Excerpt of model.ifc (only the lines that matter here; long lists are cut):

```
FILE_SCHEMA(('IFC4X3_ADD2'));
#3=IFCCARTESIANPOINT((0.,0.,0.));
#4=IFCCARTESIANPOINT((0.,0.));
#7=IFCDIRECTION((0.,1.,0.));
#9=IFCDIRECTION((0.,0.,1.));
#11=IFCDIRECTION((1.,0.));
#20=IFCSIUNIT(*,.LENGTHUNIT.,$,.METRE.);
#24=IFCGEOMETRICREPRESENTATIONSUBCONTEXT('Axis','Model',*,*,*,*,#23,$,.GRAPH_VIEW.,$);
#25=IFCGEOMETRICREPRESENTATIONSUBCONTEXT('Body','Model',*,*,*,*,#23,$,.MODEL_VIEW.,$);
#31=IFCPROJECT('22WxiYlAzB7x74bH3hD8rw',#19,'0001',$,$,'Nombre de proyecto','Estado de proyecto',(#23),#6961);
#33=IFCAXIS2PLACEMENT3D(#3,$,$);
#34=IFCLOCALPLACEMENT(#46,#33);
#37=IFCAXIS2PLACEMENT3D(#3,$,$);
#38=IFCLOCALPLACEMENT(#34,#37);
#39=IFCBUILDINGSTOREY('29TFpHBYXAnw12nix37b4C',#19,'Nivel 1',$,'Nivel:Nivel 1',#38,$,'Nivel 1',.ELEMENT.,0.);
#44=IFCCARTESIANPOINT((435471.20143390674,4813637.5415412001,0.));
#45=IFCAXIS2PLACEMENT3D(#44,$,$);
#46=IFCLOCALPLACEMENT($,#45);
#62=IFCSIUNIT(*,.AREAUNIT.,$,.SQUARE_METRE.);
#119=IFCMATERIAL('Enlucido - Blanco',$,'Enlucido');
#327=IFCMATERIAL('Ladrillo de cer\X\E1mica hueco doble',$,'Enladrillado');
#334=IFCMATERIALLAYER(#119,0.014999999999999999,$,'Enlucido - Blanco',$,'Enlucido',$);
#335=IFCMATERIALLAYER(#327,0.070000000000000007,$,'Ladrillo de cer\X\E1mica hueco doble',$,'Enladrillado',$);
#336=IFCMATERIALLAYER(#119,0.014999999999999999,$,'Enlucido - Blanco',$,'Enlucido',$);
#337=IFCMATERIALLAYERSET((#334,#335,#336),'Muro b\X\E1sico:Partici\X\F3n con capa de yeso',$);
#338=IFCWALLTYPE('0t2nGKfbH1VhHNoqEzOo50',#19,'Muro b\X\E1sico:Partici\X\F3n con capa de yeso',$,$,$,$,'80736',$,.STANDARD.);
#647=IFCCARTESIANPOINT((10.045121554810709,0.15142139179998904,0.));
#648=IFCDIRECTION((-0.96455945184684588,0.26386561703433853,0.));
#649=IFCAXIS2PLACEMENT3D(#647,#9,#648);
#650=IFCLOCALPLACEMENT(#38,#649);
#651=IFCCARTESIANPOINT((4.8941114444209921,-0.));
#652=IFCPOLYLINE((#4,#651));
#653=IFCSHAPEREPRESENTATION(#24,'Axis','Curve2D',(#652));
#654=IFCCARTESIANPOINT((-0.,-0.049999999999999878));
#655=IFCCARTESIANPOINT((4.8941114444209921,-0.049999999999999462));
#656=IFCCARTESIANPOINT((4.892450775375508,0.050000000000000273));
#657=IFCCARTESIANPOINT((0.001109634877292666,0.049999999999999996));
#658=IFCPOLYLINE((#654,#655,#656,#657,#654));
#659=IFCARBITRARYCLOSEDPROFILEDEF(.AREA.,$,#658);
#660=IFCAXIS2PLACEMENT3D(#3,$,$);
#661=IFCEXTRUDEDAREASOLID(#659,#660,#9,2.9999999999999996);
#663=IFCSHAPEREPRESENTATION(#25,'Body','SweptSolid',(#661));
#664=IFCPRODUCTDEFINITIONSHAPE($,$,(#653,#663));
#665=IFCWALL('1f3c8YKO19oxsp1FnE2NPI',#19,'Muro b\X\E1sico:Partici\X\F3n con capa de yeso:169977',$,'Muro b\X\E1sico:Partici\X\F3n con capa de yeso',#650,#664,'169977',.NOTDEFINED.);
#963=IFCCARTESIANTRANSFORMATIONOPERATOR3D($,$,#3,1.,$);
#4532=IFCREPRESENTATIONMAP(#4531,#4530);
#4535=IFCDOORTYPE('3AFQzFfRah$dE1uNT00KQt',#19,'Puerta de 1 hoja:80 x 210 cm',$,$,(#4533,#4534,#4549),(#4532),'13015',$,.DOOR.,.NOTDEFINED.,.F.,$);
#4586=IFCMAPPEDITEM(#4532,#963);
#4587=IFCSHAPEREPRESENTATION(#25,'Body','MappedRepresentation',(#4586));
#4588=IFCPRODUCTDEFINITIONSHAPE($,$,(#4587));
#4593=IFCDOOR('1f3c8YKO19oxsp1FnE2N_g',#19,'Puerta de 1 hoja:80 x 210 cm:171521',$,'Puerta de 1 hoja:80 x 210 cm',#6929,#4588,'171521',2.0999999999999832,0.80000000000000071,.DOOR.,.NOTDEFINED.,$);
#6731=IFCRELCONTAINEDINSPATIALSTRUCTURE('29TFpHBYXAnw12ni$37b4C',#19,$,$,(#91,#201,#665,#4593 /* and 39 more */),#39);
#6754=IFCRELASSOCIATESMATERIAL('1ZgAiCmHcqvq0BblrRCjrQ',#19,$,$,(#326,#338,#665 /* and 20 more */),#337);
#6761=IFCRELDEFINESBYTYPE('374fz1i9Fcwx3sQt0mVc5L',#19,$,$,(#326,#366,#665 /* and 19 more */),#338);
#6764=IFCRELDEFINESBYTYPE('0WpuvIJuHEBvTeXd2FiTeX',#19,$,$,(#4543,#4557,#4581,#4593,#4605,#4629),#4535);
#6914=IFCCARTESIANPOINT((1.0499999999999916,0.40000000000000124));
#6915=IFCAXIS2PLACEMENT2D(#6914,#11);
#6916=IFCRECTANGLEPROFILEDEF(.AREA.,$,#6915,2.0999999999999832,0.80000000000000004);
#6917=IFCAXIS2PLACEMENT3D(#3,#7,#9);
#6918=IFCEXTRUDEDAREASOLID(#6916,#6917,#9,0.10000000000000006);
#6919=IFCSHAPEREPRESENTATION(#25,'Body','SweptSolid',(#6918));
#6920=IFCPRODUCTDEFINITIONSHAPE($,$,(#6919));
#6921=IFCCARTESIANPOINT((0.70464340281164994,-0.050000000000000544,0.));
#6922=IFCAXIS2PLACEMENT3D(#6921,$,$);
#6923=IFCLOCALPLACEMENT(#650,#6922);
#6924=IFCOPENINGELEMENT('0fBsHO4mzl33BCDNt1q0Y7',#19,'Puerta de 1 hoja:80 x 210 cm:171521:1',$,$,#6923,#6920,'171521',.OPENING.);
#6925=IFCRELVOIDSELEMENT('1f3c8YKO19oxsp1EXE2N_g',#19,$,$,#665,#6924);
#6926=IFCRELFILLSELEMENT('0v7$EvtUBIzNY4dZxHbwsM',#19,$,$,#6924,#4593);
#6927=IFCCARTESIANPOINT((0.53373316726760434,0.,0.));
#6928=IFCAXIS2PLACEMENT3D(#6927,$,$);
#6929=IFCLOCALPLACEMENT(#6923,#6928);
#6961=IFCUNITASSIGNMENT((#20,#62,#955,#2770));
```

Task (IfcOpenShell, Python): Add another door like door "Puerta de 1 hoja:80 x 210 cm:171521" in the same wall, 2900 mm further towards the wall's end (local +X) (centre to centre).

```python
import ifcopenshell
import ifcopenshell.api.feature
import ifcopenshell.api.geometry
import ifcopenshell.api.root
import ifcopenshell.geom
import ifcopenshell.util.element
import ifcopenshell.util.placement
import ifcopenshell.util.shape

model = ifcopenshell.open("model.ifc")
settings = ifcopenshell.geom.settings()


def volume(element):
    """Net volume in cubic metres, openings subtracted."""
    shape = ifcopenshell.geom.create_shape(settings, element)
    return ifcopenshell.util.shape.get_volume(shape.geometry)


def reuse_history(source, copy):
    """copy_class also copies each property set's owner history, people and application; keep the originals."""
    for rel in copy.IsDefinedBy:
        if rel.is_a("IfcRelDefinesByProperties") and (history := rel.RelatingPropertyDefinition.OwnerHistory):
            rel.RelatingPropertyDefinition.OwnerHistory = source.OwnerHistory
            ifcopenshell.util.element.remove_deep2(model, history)


door = model.by_id(4593)
opening = door.FillsVoids[0].RelatingOpeningElement
wall = opening.VoidsElements[0].RelatingBuildingElement
before = volume(wall)
shift = ifcopenshell.util.placement.get_local_placement(wall.ObjectPlacement)[:3, 0] * 2.9

# copy_class copies the void relationship, type, container and properties, but no geometry.
new_opening = ifcopenshell.api.root.copy_class(model, product=opening)
new_opening.Representation = ifcopenshell.util.element.copy_deep(
    model, opening.Representation, exclude=["IfcGeometricRepresentationContext", "IfcRepresentationMap"]
)
new_opening.Name = "Puerta de 1 hoja:80 x 210 cm"
new_opening.Tag = None
new_door = ifcopenshell.api.root.copy_class(model, product=door)
new_door.Representation = ifcopenshell.util.element.copy_deep(
    model, door.Representation, exclude=["IfcGeometricRepresentationContext", "IfcRepresentationMap"]
)
new_door.Name = "Puerta de 1 hoja:80 x 210 cm"
new_door.Tag = None
reuse_history(door, new_door)
ifcopenshell.api.feature.add_filling(model, opening=new_opening, element=new_door)

for old, new in ((opening, new_opening), (door, new_door)):
    matrix = ifcopenshell.util.placement.get_local_placement(old.ObjectPlacement)
    matrix[:3, 3] += shift
    ifcopenshell.api.geometry.edit_object_placement(model, product=new, matrix=matrix, is_si=False)

after = volume(wall)

print(f"wall volume {before:.3f} -> {after:.3f} m3")

model.write("model-out.ifc")
```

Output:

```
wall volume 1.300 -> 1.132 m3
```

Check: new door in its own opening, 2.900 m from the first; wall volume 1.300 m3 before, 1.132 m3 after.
